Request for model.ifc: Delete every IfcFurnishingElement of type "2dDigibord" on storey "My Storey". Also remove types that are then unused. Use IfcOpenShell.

First a look at what the model holds.

```python
import ifcopenshell
import ifcopenshell.util.element

model = ifcopenshell.open("model.ifc")
print(model.schema)
storey = next(s for s in model.by_type("IfcBuildingStorey") if s.Name == "My Storey")
furniture = [e for e in ifcopenshell.util.element.get_decomposition(storey) if e.is_a("IfcFurnishingElement")]
seen = {}
for e in furniture:
    element_type = ifcopenshell.util.element.get_type(e)
    name = element_type.Name if element_type not in (None, e) else None
    seen[name] = seen.get(name, 0) + 1
for name, count in sorted(seen.items(), key=str):
    print(count, "x", name)
```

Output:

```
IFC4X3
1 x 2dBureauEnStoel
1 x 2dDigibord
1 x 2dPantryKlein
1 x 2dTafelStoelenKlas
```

```python
import ifcopenshell
import ifcopenshell.api.root
import ifcopenshell.util.element

model = ifcopenshell.open("model.ifc")

storey = next(s for s in model.by_type("IfcBuildingStorey") if s.Name == "My Storey")
furniture = [e for e in ifcopenshell.util.element.get_decomposition(storey) if e.is_a("IfcFurnishingElement")]
targets = [e for e in furniture if (t := ifcopenshell.util.element.get_type(e)) not in (None, e) and t.Name == "2dDigibord"]
types = {ifcopenshell.util.element.get_type(e) for e in targets} - {None, *targets}

for e in targets:
    ifcopenshell.api.root.remove_product(model, product=e)
print(len(targets), "removed")

unused = [t for t in types if not ifcopenshell.util.element.get_types(t)]
for t in unused:
    ifcopenshell.api.root.remove_product(model, product=t)
print(len(unused), "unused types removed")

model.write("model_v2.ifc")
```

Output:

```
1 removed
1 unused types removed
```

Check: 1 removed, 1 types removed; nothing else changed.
